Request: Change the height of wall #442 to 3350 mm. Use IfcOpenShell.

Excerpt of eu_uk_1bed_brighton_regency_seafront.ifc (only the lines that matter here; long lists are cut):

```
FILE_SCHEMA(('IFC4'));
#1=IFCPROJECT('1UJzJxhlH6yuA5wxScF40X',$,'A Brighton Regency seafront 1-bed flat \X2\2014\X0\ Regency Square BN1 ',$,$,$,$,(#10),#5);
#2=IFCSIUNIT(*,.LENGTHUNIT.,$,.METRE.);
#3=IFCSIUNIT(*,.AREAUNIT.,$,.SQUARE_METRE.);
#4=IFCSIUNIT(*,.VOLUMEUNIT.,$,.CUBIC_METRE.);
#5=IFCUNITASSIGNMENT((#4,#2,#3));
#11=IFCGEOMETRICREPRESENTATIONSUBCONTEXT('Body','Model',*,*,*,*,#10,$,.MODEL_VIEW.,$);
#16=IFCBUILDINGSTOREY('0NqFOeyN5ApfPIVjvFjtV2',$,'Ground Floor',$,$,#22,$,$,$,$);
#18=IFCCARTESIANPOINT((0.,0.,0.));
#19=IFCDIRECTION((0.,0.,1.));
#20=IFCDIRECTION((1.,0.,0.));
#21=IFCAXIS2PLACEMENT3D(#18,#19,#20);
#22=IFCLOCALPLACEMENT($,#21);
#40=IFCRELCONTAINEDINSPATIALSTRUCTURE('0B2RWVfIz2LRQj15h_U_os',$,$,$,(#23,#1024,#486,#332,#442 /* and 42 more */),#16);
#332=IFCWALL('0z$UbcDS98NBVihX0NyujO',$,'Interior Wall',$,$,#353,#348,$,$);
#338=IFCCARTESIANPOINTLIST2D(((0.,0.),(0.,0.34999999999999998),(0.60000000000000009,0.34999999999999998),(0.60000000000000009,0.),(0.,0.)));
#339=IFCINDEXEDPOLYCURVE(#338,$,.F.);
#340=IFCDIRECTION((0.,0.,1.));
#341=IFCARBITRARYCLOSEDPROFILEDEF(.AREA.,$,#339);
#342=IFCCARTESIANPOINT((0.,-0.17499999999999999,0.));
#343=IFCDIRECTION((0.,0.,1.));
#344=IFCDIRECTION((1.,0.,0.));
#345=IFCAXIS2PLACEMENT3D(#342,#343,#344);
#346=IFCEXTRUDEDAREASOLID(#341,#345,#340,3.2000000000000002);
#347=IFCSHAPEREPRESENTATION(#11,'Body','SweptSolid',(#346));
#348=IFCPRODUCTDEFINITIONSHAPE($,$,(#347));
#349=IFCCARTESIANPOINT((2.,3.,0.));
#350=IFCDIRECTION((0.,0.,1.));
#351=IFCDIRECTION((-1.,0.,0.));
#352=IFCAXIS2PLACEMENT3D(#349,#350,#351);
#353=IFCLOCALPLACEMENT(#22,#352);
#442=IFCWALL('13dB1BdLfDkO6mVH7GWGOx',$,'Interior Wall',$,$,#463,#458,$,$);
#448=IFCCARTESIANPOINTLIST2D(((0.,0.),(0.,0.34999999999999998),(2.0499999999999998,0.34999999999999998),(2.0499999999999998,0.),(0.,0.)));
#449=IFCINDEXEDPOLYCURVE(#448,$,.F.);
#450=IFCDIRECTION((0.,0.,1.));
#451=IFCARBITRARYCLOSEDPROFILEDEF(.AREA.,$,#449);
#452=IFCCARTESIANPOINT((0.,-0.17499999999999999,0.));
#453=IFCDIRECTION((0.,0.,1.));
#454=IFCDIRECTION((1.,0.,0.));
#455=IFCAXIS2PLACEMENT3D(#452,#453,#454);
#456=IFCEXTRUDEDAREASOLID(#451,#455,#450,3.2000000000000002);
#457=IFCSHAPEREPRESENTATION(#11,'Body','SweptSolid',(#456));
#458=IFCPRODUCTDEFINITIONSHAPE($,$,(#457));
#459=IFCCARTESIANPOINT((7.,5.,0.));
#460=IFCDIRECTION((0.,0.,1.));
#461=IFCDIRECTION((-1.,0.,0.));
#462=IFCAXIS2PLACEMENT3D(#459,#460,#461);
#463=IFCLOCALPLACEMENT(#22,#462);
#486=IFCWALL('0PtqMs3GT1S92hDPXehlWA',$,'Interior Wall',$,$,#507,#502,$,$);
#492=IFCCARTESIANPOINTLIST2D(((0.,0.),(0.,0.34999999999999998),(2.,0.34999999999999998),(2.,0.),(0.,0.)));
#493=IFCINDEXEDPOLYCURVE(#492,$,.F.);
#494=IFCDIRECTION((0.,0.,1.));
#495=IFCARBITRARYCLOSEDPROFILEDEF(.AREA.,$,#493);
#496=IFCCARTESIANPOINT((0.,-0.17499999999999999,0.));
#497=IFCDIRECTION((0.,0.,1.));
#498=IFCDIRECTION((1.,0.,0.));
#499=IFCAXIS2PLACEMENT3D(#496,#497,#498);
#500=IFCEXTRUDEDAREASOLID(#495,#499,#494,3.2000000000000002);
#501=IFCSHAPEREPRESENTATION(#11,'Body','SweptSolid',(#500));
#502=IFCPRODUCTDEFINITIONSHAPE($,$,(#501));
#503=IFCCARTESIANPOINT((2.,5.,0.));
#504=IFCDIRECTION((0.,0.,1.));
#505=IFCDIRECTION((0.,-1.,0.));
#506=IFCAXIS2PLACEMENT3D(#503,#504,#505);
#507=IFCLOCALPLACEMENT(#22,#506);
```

```python
import ifcopenshell
import ifcopenshell.geom
import ifcopenshell.util.representation
import ifcopenshell.util.shape

model = ifcopenshell.open("eu_uk_1bed_brighton_regency_seafront.ifc")
settings = ifcopenshell.geom.settings()


def volume(element):
    """Net volume in cubic metres, openings subtracted."""
    shape = ifcopenshell.geom.create_shape(settings, element)
    return ifcopenshell.util.shape.get_volume(shape.geometry)


wall = model.by_guid("13dB1BdLfDkO6mVH7GWGOx")
before = volume(wall)

body = ifcopenshell.util.representation.get_representation(wall, "Model", "Body")
solid = body.Items[0]
old_height = solid.Depth
solid.Depth = 3.35
after = volume(wall)

print(f"height {old_height:g} -> {solid.Depth:g}, volume {before:.3f} -> {after:.3f} m3")

model.write("eu_uk_1bed_brighton_regency_seafront_edited.ifc")
```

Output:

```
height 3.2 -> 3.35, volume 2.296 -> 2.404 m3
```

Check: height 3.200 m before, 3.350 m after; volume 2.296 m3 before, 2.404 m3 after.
